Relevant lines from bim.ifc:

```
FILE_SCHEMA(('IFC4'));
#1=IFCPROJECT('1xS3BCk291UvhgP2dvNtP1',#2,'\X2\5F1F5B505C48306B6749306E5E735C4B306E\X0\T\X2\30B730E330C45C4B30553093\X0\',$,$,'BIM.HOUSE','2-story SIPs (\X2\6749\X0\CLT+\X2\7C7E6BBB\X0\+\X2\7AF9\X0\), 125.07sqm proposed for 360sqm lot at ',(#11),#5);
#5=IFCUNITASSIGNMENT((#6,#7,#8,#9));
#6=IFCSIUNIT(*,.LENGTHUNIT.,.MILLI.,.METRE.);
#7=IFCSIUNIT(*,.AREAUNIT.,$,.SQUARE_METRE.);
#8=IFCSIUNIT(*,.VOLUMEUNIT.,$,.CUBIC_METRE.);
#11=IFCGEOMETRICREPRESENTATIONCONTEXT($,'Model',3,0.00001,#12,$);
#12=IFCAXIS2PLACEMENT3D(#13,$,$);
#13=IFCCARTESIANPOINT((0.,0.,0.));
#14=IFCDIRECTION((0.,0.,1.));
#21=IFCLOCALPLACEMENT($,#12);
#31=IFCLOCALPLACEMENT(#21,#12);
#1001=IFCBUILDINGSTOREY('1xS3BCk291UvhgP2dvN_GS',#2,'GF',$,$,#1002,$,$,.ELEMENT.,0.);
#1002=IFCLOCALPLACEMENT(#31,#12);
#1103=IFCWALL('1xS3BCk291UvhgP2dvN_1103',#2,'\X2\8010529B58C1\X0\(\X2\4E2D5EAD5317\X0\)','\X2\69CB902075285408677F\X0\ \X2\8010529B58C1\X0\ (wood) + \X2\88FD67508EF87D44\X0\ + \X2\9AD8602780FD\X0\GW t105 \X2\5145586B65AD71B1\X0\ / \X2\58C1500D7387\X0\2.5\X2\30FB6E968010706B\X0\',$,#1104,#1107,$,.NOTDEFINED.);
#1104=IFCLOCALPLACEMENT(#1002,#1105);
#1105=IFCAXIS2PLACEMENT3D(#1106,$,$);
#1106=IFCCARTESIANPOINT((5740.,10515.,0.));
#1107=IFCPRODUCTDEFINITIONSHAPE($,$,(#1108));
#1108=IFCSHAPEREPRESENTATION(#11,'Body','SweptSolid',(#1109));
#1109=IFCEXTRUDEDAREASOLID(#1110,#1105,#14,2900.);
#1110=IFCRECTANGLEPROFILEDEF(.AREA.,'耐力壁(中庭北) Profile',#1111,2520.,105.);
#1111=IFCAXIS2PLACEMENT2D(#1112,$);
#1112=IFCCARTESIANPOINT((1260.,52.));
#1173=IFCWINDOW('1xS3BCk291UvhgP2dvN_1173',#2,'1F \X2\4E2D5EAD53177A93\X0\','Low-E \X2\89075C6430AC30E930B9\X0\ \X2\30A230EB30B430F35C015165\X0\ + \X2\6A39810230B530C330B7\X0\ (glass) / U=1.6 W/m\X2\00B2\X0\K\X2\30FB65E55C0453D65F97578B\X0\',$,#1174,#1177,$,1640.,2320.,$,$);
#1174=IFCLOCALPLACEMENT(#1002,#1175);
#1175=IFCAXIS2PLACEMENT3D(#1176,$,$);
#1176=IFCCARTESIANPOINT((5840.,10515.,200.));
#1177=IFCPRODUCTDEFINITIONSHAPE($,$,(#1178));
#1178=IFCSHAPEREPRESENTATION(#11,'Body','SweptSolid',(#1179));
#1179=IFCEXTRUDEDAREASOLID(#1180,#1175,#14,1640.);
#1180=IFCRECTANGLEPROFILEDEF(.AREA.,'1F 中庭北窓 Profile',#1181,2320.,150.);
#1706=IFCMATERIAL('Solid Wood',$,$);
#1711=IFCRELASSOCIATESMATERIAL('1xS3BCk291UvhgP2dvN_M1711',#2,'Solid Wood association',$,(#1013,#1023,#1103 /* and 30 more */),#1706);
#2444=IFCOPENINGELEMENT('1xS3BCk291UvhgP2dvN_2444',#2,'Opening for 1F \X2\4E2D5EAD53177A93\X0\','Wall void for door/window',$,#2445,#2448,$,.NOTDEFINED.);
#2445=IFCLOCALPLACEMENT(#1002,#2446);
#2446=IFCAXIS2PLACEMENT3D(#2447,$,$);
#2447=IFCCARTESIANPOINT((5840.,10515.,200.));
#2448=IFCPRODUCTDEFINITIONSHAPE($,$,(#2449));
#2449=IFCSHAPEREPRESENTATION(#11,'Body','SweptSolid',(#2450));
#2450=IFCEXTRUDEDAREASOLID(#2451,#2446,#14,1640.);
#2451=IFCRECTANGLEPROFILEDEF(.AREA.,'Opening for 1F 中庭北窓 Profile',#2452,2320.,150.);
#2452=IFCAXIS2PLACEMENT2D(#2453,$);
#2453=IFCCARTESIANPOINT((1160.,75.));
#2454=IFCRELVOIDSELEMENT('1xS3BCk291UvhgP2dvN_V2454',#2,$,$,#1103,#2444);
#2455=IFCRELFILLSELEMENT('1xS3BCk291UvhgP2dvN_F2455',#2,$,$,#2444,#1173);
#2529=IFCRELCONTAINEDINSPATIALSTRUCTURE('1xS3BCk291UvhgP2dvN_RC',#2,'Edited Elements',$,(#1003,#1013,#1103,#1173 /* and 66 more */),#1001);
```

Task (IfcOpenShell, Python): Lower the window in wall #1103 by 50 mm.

```python
import numpy as np
import ifcopenshell
import ifcopenshell.api.geometry
import ifcopenshell.util.placement
import ifcopenshell.util.unit

model = ifcopenshell.open("bim.ifc")
unit_scale = ifcopenshell.util.unit.calculate_unit_scale(model)

window = model.by_id(1173)
opening = window.FillsVoids[0].RelatingOpeningElement
dz = -0.05 / unit_scale

shift = np.array([0.0, 0.0, dz])
# The window is not placed relative to its opening, so move both.
for product in (opening, window):
    matrix = ifcopenshell.util.placement.get_local_placement(product.ObjectPlacement)
    matrix[:3, 3] += shift
    ifcopenshell.api.geometry.edit_object_placement(model, product=product, matrix=matrix, is_si=False)

print(f"moved by {dz * unit_scale:+.3f} m")

model.write("bim_rev.ifc")
```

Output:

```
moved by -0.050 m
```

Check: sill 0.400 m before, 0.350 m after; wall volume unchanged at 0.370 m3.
